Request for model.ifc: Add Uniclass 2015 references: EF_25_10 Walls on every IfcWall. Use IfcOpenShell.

First a look at what the model holds.

```python
import ifcopenshell

model = ifcopenshell.open("model.ifc")
print(model.schema)
print("classifications:", [c.Name for c in model.by_type("IfcClassification")])
for ifc_class in ("IfcDoor", "IfcRoof", "IfcStair", "IfcWall", "IfcWindow"):
    print(ifc_class, len(model.by_type(ifc_class)))
```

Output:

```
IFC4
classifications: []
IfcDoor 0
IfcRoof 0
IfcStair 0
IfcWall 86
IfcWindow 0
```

```python
import ifcopenshell
import ifcopenshell.api.classification

model = ifcopenshell.open("model.ifc")

system = ifcopenshell.api.classification.add_classification(model, classification="Uniclass 2015")

codes = {
    "IfcWall": ("EF_25_10", "Walls"),
}
for ifc_class, (code, name) in codes.items():
    products = model.by_type(ifc_class)
    ifcopenshell.api.classification.add_reference(
        model, products=products, classification=system, identification=code, name=name
    )
    print(code, len(products))

model.write("model-out.ifc")
```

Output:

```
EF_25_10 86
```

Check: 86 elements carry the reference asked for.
